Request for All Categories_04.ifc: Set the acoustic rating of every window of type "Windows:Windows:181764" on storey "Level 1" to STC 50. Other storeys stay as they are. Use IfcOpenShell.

First a look at what the model holds.

```python
import ifcopenshell
import ifcopenshell.util.element

model = ifcopenshell.open("All Categories_04.ifc")
print(model.schema)
storey = next(s for s in model.by_type("IfcBuildingStorey") if s.Name == "Level 1")
windows = [e for e in ifcopenshell.util.element.get_decomposition(storey) if e.is_a("IfcWindow")]
seen = {}
for e in windows:
    element_type = ifcopenshell.util.element.get_type(e)
    key = (element_type.Name if element_type != e and element_type else None, ifcopenshell.util.element.get_pset(e, "Pset_WindowCommon", "AcousticRating"))
    seen[key] = seen.get(key, 0) + 1
for (name, value), count in sorted(seen.items(), key=str):
    print(count, "x", name, "|", value)
```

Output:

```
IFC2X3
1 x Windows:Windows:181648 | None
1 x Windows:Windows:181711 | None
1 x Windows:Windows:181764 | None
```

```python
import ifcopenshell
import ifcopenshell.api.pset
import ifcopenshell.util.element

model = ifcopenshell.open("All Categories_04.ifc")

storey = next(s for s in model.by_type("IfcBuildingStorey") if s.Name == "Level 1")
windows = [e for e in ifcopenshell.util.element.get_decomposition(storey) if e.is_a("IfcWindow")]

count = 0
for e in windows:
    element_type = ifcopenshell.util.element.get_type(e)
    if element_type in (None, e) or element_type.Name != "Windows:Windows:181764":
        continue
    # add_pset returns the element's existing set when there is one.
    pset = ifcopenshell.api.pset.add_pset(model, product=e, name="Pset_WindowCommon")
    ifcopenshell.api.pset.edit_pset(model, pset=pset, properties={"AcousticRating": "STC 50"})
    count += 1

print(count, "windows updated")

model.write("All Categories_04_v2.ifc")
```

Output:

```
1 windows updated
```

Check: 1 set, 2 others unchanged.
